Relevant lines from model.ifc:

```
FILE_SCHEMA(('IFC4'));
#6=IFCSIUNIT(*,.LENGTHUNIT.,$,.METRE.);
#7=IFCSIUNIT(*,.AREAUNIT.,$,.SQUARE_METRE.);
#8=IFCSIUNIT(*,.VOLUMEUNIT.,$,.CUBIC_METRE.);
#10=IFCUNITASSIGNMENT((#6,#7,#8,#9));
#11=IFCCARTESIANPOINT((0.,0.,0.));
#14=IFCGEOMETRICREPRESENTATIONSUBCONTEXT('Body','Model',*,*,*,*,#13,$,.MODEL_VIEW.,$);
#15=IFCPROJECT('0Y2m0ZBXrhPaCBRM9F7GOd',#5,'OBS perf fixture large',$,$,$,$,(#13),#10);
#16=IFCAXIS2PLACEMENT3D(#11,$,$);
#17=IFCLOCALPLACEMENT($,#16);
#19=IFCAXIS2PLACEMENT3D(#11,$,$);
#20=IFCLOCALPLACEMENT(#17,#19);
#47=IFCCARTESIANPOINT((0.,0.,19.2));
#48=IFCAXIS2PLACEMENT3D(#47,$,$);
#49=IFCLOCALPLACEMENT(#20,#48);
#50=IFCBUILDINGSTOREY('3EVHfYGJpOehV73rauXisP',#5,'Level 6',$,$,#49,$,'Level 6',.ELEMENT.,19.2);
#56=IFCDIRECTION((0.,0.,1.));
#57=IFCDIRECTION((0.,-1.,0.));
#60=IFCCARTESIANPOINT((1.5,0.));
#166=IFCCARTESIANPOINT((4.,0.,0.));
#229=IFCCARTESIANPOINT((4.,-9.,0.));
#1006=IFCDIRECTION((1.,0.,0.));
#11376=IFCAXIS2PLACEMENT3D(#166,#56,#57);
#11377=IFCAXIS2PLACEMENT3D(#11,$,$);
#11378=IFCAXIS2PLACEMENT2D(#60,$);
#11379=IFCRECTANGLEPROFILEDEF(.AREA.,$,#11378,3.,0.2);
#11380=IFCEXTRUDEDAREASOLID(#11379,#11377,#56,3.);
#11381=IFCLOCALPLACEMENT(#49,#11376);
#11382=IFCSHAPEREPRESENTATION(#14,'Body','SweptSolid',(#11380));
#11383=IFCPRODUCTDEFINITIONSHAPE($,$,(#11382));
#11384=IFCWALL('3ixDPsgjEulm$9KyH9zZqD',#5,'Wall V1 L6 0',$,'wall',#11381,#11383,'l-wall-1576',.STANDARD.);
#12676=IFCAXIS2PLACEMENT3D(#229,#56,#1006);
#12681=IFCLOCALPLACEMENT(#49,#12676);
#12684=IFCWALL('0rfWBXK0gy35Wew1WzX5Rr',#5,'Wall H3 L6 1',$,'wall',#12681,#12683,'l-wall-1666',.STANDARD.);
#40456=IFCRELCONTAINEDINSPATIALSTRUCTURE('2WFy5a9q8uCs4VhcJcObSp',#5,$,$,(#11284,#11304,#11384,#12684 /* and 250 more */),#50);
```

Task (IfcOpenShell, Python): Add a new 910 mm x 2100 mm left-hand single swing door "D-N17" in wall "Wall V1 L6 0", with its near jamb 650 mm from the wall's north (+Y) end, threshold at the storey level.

```python
import numpy as np
import ifcopenshell
import ifcopenshell.api.feature
import ifcopenshell.api.geometry
import ifcopenshell.api.root
import ifcopenshell.api.spatial
import ifcopenshell.geom
import ifcopenshell.util.element
import ifcopenshell.util.placement
import ifcopenshell.util.representation
import ifcopenshell.util.shape
import ifcopenshell.util.unit

model = ifcopenshell.open("model.ifc")
unit_scale = ifcopenshell.util.unit.calculate_unit_scale(model)
settings = ifcopenshell.geom.settings()


def volume(element):
    """Net volume in cubic metres, openings subtracted."""
    shape = ifcopenshell.geom.create_shape(settings, element)
    return ifcopenshell.util.shape.get_volume(shape.geometry)


wall = model.by_id(11384)
storey = ifcopenshell.util.element.get_container(wall, ifc_class="IfcBuildingStorey")
context = ifcopenshell.util.representation.get_context(model, "Model", "Body", "MODEL_VIEW")
before = volume(wall)

width, height, from_end, sill = 0.91, 2.1, 0.65, 0.0  # metres

# The wall runs along its own X axis, and the end named is its -X end.
wall_shape = ifcopenshell.geom.create_shape(settings, wall)
x, y, z = ifcopenshell.util.shape.get_vertices(wall_shape.geometry).T
start = x.min() + from_end
face, thickness = float(y.min()), float(y.max() - y.min())
wall_matrix = ifcopenshell.util.placement.get_local_placement(wall.ObjectPlacement)
level = ifcopenshell.util.placement.get_local_placement(storey.ObjectPlacement)[2, 3]


def in_wall(x, y):
    """Placement at x, y metres in the wall's axes, at sill height."""
    matrix = wall_matrix.copy()
    matrix[:, 3] = wall_matrix @ np.array([x / unit_scale, y / unit_scale, 0.0, 1.0])
    matrix[2, 3] = level + sill / unit_scale
    return matrix


# Opening: a box that overshoots both wall faces by 50 mm.
opening = ifcopenshell.api.root.create_entity(model, ifc_class="IfcOpeningElement", predefined_type="OPENING")
box = ifcopenshell.api.geometry.add_wall_representation(
    model, context=context, length=width, height=height, thickness=thickness + 0.1
)
ifcopenshell.api.geometry.assign_representation(model, product=opening, representation=box)
ifcopenshell.api.geometry.edit_object_placement(model, product=opening, matrix=in_wall(start, face - 0.05), is_si=False)
ifcopenshell.api.feature.add_feature(model, feature=opening, element=wall)

door = ifcopenshell.api.root.create_entity(model, ifc_class="IfcDoor", name="D-N17", predefined_type="DOOR")
door.OverallWidth, door.OverallHeight = width / unit_scale, height / unit_scale
door.OperationType = "SINGLE_SWING_LEFT"
body = ifcopenshell.api.geometry.add_door_representation(
    model,
    context=context,
    overall_width=door.OverallWidth,
    overall_height=door.OverallHeight,
    operation_type="SINGLE_SWING_LEFT",
    lining_properties={"LiningDepth": thickness / unit_scale, "ThresholdDepth": thickness / unit_scale},
)
ifcopenshell.api.geometry.assign_representation(model, product=door, representation=body)
ifcopenshell.api.spatial.assign_container(model, products=[door], relating_structure=storey)
ifcopenshell.api.feature.add_filling(model, opening=opening, element=door)

# The lining spans the wall, so the door starts at the wall face.
ifcopenshell.api.geometry.edit_object_placement(model, product=door, matrix=in_wall(start, face), is_si=False)

after = volume(wall)

print(f"wall volume {before:.3f} -> {after:.3f} m3")

model.write("model_rev.ifc")
```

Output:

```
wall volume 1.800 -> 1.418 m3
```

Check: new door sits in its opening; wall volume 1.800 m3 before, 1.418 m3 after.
